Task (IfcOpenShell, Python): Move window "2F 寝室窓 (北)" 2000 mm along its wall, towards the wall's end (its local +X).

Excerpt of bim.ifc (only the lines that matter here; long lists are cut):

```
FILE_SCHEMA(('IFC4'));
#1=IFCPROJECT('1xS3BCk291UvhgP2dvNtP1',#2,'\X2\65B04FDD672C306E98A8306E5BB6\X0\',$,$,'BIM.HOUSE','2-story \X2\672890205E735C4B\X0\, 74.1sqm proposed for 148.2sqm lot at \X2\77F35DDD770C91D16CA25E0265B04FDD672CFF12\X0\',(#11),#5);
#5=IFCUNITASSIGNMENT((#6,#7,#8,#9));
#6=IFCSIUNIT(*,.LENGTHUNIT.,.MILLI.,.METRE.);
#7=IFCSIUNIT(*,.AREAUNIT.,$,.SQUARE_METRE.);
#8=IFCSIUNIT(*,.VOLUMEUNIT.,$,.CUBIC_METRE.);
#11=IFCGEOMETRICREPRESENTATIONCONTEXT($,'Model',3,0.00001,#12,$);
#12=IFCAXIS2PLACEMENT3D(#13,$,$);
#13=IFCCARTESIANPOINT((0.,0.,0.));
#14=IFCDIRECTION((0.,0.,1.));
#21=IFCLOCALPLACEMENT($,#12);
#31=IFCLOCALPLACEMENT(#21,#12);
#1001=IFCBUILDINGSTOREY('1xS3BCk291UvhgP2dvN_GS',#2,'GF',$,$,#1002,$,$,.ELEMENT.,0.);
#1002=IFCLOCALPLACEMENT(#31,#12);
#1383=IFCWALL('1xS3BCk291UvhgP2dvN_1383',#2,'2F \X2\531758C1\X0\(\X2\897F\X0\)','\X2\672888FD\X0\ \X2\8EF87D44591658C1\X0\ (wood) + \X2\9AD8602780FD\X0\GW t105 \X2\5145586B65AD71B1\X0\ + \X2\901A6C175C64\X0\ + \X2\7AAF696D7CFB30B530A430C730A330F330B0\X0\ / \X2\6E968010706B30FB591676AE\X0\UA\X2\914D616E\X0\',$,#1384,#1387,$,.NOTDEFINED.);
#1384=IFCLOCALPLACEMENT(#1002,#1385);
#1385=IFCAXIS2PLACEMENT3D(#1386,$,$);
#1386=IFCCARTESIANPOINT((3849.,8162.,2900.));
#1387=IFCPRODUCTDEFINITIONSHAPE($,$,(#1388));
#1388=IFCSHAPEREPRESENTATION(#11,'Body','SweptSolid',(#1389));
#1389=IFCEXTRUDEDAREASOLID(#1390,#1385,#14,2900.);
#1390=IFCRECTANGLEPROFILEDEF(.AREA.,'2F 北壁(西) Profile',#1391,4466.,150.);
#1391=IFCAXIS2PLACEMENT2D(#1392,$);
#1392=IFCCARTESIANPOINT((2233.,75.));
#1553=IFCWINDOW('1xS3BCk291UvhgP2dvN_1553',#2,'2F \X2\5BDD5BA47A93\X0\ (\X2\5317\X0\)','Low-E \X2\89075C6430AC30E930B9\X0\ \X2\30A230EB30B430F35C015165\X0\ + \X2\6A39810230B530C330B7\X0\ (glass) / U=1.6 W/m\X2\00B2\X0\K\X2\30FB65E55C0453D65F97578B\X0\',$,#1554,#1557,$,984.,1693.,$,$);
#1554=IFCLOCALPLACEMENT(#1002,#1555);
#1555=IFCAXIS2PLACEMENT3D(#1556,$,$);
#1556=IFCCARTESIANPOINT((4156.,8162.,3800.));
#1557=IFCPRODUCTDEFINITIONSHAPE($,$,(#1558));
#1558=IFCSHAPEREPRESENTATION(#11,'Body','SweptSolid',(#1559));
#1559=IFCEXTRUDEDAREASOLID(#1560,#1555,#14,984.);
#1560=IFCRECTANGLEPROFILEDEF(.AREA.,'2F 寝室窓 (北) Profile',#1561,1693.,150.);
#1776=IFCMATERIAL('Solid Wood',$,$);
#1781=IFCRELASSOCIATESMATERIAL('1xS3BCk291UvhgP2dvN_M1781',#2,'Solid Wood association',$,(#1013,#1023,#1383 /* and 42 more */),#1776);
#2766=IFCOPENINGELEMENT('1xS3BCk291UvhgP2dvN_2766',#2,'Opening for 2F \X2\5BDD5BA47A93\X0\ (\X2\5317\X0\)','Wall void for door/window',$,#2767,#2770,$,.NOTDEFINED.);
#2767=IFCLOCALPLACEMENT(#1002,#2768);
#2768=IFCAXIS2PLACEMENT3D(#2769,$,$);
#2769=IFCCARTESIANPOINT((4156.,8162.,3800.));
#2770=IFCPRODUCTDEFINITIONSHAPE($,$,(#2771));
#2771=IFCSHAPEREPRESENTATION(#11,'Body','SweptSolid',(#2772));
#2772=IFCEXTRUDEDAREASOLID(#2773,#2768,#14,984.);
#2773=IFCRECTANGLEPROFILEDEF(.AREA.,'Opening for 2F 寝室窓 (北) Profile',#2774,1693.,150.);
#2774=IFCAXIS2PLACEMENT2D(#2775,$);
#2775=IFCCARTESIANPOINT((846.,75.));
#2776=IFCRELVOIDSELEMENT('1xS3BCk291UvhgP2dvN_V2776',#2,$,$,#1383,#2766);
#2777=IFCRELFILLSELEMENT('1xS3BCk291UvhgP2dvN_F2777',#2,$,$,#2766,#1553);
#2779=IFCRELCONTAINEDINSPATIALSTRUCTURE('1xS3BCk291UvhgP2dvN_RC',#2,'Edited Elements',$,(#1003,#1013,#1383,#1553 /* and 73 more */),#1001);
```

```python
import ifcopenshell
import ifcopenshell.api.geometry
import ifcopenshell.util.placement

model = ifcopenshell.open("bim.ifc")

window = model.by_guid("1xS3BCk291UvhgP2dvN_1553")
opening = window.FillsVoids[0].RelatingOpeningElement
wall = opening.VoidsElements[0].RelatingBuildingElement

wall_matrix = ifcopenshell.util.placement.get_local_placement(wall.ObjectPlacement)
shift = wall_matrix[:3, 0] * 2000.0
before = ifcopenshell.util.placement.get_local_placement(window.ObjectPlacement)[:3, 3].copy()

# The window is not placed relative to its opening, so move both.
for product in (opening, window):
    matrix = ifcopenshell.util.placement.get_local_placement(product.ObjectPlacement)
    matrix[:3, 3] += shift
    ifcopenshell.api.geometry.edit_object_placement(model, product=product, matrix=matrix, is_si=False)

after = ifcopenshell.util.placement.get_local_placement(window.ObjectPlacement)[:3, 3]
print("window moved by", (after - before).round(3) + 0.0)

model.write("bim_v2.ifc")
```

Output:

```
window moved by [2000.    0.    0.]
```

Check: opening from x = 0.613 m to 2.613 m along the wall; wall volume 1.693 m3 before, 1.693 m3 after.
